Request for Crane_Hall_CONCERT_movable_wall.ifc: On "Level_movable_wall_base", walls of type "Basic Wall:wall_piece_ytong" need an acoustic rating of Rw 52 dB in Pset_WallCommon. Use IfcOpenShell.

First a look at what the model holds.

```python
import ifcopenshell
import ifcopenshell.util.element

model = ifcopenshell.open("Crane_Hall_CONCERT_movable_wall.ifc")
print(model.schema)
storey = next(s for s in model.by_type("IfcBuildingStorey") if s.Name == "Level_movable_wall_base")
walls = [e for e in ifcopenshell.util.element.get_decomposition(storey) if e.is_a("IfcWall")]
seen = {}
for e in walls:
    element_type = ifcopenshell.util.element.get_type(e)
    key = (element_type.Name if element_type != e and element_type else None, ifcopenshell.util.element.get_pset(e, "Pset_WallCommon", "AcousticRating"))
    seen[key] = seen.get(key, 0) + 1
for (name, value), count in sorted(seen.items(), key=str):
    print(count, "x", name, "|", value)
```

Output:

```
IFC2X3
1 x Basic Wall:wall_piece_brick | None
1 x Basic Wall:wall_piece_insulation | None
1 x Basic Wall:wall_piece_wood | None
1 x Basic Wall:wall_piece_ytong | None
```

```python
import ifcopenshell
import ifcopenshell.api.pset
import ifcopenshell.util.element

model = ifcopenshell.open("Crane_Hall_CONCERT_movable_wall.ifc")

storey = next(s for s in model.by_type("IfcBuildingStorey") if s.Name == "Level_movable_wall_base")
walls = [e for e in ifcopenshell.util.element.get_decomposition(storey) if e.is_a("IfcWall")]

count = 0
for e in walls:
    element_type = ifcopenshell.util.element.get_type(e)
    if element_type in (None, e) or element_type.Name != "Basic Wall:wall_piece_ytong":
        continue
    # add_pset returns the element's existing set when there is one.
    pset = ifcopenshell.api.pset.add_pset(model, product=e, name="Pset_WallCommon")
    ifcopenshell.api.pset.edit_pset(model, pset=pset, properties={"AcousticRating": "Rw 52 dB"})
    count += 1

print(count, "walls updated")

model.write("Crane_Hall_CONCERT_movable_wall_v2.ifc")
```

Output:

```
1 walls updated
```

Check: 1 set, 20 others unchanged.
